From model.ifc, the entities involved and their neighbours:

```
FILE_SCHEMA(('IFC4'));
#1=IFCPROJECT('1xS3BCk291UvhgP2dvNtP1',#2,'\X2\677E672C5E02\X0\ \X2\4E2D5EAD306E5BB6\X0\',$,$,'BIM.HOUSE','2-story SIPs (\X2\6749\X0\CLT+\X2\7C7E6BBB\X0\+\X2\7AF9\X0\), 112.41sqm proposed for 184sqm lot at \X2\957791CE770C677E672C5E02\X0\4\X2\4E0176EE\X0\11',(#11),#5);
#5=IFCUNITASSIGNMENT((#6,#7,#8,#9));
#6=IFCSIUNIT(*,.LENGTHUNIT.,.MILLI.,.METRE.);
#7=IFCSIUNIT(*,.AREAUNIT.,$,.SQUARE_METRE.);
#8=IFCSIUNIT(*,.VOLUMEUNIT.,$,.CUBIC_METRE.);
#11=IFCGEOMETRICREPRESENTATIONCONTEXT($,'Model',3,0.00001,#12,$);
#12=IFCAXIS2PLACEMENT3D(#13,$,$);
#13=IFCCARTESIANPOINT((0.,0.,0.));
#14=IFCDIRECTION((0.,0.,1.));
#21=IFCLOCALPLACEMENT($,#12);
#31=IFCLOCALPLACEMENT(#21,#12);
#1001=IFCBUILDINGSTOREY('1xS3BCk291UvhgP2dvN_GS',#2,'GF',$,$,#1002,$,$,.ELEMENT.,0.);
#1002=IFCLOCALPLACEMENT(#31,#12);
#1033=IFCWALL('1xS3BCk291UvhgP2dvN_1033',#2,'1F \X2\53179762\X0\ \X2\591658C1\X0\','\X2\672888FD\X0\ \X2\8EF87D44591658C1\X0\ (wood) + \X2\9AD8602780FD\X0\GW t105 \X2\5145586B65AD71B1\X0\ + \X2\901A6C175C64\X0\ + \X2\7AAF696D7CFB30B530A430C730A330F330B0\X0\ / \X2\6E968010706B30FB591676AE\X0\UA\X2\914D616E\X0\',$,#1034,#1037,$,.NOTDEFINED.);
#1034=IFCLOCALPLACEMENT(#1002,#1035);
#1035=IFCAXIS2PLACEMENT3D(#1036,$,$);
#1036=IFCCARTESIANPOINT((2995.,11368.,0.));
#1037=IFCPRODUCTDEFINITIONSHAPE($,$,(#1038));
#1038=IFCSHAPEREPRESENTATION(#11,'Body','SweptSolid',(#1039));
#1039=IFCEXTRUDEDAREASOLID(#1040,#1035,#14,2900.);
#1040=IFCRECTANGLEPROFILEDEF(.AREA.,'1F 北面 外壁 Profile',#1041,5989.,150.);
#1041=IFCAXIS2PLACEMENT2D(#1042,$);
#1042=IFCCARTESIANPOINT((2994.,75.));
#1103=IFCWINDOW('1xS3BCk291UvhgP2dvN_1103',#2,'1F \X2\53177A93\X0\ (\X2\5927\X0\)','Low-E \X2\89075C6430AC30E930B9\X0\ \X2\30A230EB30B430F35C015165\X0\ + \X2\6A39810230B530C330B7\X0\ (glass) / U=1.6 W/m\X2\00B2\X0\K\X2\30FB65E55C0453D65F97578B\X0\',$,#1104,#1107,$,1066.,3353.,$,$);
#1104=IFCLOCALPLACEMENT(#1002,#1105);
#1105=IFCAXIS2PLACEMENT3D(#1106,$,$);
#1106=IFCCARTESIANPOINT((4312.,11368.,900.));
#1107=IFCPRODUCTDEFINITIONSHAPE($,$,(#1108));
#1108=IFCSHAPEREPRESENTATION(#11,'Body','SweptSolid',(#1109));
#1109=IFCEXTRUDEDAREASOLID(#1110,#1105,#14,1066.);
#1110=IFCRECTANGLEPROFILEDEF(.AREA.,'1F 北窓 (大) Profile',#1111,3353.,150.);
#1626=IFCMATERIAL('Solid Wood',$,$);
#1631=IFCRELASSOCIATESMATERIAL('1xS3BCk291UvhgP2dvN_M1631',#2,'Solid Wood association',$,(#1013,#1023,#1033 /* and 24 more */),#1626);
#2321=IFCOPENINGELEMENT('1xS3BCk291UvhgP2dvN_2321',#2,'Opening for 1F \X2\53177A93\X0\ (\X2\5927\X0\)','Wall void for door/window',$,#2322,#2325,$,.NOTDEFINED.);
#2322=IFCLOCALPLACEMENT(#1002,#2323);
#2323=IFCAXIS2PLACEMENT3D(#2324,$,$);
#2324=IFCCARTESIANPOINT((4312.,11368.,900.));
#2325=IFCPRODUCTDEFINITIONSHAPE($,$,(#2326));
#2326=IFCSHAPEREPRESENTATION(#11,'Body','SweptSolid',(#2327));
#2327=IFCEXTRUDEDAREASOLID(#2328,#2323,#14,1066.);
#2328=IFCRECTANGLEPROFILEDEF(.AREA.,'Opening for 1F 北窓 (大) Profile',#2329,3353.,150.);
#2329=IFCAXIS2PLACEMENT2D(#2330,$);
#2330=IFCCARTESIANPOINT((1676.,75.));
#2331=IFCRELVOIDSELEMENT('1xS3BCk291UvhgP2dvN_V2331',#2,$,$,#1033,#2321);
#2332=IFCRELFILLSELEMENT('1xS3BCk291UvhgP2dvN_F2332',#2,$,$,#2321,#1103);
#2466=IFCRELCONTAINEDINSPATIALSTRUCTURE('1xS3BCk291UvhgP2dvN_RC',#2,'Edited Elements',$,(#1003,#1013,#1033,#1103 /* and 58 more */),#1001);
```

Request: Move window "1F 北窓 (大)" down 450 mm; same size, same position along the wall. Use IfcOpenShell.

```python
import numpy as np
import ifcopenshell
import ifcopenshell.api.geometry
import ifcopenshell.util.placement
import ifcopenshell.util.unit

model = ifcopenshell.open("model.ifc")
unit_scale = ifcopenshell.util.unit.calculate_unit_scale(model)

window = model.by_guid("1xS3BCk291UvhgP2dvN_1103")
opening = window.FillsVoids[0].RelatingOpeningElement
dz = -450.0

shift = np.array([0.0, 0.0, dz])
# The window is not placed relative to its opening, so move both.
for product in (opening, window):
    matrix = ifcopenshell.util.placement.get_local_placement(product.ObjectPlacement)
    matrix[:3, 3] += shift
    ifcopenshell.api.geometry.edit_object_placement(model, product=product, matrix=matrix, is_si=False)

print(f"moved by {dz * unit_scale:+.3f} m")

model.write("model_updated.ifc")
```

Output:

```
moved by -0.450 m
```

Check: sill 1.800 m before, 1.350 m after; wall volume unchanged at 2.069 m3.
